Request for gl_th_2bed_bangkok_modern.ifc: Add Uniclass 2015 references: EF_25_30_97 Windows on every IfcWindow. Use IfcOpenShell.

First a look at what the model holds.

```python
import ifcopenshell

model = ifcopenshell.open("gl_th_2bed_bangkok_modern.ifc")
print(model.schema)
print("classifications:", [c.Name for c in model.by_type("IfcClassification")])
for ifc_class in ("IfcDoor", "IfcRoof", "IfcStair", "IfcWall", "IfcWindow"):
    print(ifc_class, len(model.by_type(ifc_class)))
```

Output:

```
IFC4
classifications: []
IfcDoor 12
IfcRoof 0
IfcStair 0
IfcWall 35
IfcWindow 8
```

```python
import ifcopenshell
import ifcopenshell.api.classification

model = ifcopenshell.open("gl_th_2bed_bangkok_modern.ifc")

system = ifcopenshell.api.classification.add_classification(model, classification="Uniclass 2015")

codes = {
    "IfcWindow": ("EF_25_30_97", "Windows"),
}
for ifc_class, (code, name) in codes.items():
    products = model.by_type(ifc_class)
    ifcopenshell.api.classification.add_reference(
        model, products=products, classification=system, identification=code, name=name
    )
    print(code, len(products))

model.write("gl_th_2bed_bangkok_modern-out.ifc")
```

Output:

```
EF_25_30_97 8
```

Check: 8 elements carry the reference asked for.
